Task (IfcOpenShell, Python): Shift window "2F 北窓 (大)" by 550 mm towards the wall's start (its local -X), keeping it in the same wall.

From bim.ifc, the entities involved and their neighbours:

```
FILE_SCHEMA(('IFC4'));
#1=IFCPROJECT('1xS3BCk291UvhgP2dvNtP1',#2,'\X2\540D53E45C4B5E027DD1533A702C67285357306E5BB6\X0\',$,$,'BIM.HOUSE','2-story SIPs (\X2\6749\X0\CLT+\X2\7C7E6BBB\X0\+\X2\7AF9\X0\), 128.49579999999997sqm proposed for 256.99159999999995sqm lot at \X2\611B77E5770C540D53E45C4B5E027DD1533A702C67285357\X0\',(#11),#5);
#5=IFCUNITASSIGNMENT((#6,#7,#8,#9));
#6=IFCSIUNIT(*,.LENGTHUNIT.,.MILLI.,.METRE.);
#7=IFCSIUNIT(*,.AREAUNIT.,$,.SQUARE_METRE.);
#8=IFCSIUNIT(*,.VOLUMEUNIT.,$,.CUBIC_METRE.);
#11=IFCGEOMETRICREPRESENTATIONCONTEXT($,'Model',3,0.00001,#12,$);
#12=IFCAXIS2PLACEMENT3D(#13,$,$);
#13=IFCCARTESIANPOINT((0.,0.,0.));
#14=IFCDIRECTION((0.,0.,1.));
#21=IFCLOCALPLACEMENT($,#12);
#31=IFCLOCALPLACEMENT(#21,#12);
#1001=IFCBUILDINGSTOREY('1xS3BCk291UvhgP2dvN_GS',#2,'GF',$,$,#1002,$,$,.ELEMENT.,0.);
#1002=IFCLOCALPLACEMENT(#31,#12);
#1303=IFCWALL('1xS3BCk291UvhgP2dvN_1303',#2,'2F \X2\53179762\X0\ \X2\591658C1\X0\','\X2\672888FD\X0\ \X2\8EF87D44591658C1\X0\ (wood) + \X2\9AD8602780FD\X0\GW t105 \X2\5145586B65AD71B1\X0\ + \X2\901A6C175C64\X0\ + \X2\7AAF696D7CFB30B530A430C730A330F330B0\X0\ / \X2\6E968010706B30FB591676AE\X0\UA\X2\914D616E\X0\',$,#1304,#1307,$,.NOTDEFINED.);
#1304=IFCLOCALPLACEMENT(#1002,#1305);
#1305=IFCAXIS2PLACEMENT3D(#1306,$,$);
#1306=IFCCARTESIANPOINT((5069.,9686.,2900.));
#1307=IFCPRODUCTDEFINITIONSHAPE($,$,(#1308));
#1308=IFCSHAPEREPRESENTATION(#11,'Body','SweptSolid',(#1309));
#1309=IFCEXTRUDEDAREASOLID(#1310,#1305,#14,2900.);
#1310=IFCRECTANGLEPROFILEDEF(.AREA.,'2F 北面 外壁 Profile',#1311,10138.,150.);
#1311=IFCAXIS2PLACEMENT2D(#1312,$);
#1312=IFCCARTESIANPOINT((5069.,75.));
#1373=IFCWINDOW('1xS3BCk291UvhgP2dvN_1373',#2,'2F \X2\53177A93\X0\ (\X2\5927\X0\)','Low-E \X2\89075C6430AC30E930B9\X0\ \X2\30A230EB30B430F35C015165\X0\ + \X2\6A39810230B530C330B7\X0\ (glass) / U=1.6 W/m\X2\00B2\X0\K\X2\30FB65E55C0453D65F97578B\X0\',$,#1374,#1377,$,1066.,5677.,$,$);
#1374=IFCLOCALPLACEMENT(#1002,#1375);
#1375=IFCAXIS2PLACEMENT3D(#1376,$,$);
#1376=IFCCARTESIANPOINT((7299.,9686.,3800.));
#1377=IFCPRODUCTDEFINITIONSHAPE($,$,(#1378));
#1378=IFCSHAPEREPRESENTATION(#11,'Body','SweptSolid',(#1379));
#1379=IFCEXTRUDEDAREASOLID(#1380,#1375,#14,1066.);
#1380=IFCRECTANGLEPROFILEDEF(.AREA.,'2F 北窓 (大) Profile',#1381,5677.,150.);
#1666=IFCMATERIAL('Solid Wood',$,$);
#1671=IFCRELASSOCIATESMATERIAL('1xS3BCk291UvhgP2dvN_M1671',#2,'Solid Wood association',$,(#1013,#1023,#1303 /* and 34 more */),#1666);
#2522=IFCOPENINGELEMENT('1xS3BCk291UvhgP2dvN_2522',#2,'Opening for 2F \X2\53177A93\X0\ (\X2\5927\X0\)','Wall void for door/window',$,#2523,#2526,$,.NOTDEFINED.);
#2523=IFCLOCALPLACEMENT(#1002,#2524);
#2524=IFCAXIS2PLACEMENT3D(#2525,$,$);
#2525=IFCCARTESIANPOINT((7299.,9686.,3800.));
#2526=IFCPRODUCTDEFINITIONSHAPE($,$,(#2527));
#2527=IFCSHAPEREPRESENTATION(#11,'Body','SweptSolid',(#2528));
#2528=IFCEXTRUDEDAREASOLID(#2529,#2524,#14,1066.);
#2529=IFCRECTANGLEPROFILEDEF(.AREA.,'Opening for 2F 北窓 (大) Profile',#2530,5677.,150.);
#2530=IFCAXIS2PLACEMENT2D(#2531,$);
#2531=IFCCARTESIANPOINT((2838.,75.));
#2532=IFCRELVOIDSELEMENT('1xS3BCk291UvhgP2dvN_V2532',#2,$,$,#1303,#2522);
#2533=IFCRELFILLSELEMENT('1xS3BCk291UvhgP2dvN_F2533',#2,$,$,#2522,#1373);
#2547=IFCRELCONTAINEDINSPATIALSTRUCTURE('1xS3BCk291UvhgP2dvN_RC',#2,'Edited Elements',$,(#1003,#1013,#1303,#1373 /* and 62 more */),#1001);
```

```python
import ifcopenshell
import ifcopenshell.api.geometry
import ifcopenshell.util.placement

model = ifcopenshell.open("bim.ifc")

window = model.by_guid("1xS3BCk291UvhgP2dvN_1373")
opening = window.FillsVoids[0].RelatingOpeningElement
wall = opening.VoidsElements[0].RelatingBuildingElement

wall_matrix = ifcopenshell.util.placement.get_local_placement(wall.ObjectPlacement)
shift = wall_matrix[:3, 0] * -550.0
before = ifcopenshell.util.placement.get_local_placement(window.ObjectPlacement)[:3, 3].copy()

# The window is not placed relative to its opening, so move both.
for product in (opening, window):
    matrix = ifcopenshell.util.placement.get_local_placement(product.ObjectPlacement)
    matrix[:3, 3] += shift
    ifcopenshell.api.geometry.edit_object_placement(model, product=product, matrix=matrix, is_si=False)

after = ifcopenshell.util.placement.get_local_placement(window.ObjectPlacement)[:3, 3]
print("window moved by", (after - before).round(3) + 0.0)

model.write("bim-out.ifc")
```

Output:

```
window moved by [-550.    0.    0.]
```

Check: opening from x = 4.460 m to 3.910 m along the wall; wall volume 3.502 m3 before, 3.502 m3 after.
